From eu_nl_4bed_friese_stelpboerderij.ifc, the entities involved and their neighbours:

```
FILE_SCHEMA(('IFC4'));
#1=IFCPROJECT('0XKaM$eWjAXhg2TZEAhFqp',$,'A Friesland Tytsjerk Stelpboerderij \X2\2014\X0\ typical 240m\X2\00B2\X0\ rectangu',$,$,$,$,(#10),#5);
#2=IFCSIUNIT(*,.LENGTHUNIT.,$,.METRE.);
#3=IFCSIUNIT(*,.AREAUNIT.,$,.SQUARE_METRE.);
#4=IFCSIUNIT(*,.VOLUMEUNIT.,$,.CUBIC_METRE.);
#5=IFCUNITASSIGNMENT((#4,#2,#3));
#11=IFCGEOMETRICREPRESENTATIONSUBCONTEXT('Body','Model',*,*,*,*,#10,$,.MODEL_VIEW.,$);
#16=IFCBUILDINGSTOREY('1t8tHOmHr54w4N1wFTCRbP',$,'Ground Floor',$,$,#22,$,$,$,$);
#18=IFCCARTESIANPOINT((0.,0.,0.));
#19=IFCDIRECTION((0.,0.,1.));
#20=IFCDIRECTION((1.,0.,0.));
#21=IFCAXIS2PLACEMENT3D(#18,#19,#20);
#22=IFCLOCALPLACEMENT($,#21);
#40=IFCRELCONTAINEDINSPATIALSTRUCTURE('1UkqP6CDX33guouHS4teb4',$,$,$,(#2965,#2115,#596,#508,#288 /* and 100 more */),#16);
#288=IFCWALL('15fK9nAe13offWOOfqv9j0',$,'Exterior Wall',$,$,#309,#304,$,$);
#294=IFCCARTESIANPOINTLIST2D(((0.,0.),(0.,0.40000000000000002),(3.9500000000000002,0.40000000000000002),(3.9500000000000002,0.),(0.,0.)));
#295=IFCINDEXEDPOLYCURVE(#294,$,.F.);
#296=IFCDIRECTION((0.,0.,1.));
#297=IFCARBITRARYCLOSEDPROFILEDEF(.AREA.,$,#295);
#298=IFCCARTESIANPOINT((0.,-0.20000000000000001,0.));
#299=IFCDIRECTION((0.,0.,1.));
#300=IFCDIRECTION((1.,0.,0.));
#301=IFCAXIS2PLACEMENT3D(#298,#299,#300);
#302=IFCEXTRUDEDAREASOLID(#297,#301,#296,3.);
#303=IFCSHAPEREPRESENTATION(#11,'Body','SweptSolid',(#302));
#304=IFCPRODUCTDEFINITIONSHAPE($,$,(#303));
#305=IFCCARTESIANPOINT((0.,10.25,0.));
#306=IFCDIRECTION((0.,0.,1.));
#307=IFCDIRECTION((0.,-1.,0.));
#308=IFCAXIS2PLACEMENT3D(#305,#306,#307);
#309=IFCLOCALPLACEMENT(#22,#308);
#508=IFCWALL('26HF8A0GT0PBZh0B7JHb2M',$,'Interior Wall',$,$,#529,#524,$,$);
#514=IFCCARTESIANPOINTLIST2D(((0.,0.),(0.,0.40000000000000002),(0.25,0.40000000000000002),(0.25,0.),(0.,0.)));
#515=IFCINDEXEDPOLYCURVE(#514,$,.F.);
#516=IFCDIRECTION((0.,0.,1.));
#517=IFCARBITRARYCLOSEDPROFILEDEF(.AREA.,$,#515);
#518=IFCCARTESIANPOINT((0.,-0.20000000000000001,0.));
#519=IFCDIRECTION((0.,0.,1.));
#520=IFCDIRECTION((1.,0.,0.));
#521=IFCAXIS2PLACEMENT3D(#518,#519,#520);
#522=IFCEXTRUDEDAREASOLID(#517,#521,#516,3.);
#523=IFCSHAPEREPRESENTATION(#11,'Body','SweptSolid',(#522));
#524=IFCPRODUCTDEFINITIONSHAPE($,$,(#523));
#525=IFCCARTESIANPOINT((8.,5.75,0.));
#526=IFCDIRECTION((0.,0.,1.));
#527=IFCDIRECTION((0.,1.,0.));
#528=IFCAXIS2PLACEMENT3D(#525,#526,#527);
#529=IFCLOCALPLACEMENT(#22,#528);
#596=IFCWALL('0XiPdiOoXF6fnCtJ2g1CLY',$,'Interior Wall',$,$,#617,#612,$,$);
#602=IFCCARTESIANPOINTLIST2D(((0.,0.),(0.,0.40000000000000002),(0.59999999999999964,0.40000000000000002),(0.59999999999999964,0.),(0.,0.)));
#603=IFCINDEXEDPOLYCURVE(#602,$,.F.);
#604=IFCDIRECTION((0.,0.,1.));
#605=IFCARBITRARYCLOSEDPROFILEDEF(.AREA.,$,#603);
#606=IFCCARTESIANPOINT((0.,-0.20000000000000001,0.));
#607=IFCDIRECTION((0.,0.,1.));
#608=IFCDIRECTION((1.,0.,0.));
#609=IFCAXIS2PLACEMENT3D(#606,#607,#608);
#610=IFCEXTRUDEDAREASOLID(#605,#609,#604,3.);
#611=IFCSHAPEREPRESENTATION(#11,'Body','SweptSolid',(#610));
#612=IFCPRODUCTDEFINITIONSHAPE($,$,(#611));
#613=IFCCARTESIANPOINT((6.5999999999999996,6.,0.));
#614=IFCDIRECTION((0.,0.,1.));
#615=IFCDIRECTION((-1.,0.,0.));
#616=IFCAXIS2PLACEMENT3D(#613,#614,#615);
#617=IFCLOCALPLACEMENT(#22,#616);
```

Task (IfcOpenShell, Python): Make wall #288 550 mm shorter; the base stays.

```python
import ifcopenshell
import ifcopenshell.geom
import ifcopenshell.util.representation
import ifcopenshell.util.shape
import ifcopenshell.util.unit

model = ifcopenshell.open("eu_nl_4bed_friese_stelpboerderij.ifc")
unit_scale = ifcopenshell.util.unit.calculate_unit_scale(model)
settings = ifcopenshell.geom.settings()


def volume(element):
    """Net volume in cubic metres, openings subtracted."""
    shape = ifcopenshell.geom.create_shape(settings, element)
    return ifcopenshell.util.shape.get_volume(shape.geometry)


wall = model.by_id(288)
before = volume(wall)

body = ifcopenshell.util.representation.get_representation(wall, "Model", "Body")
solid = body.Items[0]
old_height = solid.Depth
solid.Depth -= 0.55 / unit_scale
after = volume(wall)

print(f"height {old_height:g} -> {solid.Depth:g}, volume {before:.3f} -> {after:.3f} m3")

model.write("eu_nl_4bed_friese_stelpboerderij_edited.ifc")
```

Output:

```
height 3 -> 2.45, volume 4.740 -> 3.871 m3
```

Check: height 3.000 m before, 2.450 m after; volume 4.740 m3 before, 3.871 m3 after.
